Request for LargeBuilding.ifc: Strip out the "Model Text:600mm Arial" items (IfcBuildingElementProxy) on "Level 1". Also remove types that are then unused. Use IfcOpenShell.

First a look at what the model holds.

```python
import ifcopenshell
import ifcopenshell.util.element

model = ifcopenshell.open("LargeBuilding.ifc")
print(model.schema)
storey = next(s for s in model.by_type("IfcBuildingStorey") if s.Name == "Level 1")
proxies = [e for e in ifcopenshell.util.element.get_decomposition(storey) if e.is_a("IfcBuildingElementProxy")]
seen = {}
for e in proxies:
    element_type = ifcopenshell.util.element.get_type(e)
    name = element_type.Name if element_type not in (None, e) else None
    seen[name] = seen.get(name, 0) + 1
for name, count in sorted(seen.items(), key=str):
    print(count, "x", name)
```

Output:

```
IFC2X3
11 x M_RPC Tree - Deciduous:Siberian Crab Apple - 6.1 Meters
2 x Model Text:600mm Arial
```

```python
import ifcopenshell
import ifcopenshell.api.root
import ifcopenshell.util.element

model = ifcopenshell.open("LargeBuilding.ifc")

storey = next(s for s in model.by_type("IfcBuildingStorey") if s.Name == "Level 1")
proxies = [e for e in ifcopenshell.util.element.get_decomposition(storey) if e.is_a("IfcBuildingElementProxy")]
targets = [e for e in proxies if (t := ifcopenshell.util.element.get_type(e)) not in (None, e) and t.Name == "Model Text:600mm Arial"]
types = {ifcopenshell.util.element.get_type(e) for e in targets} - {None, *targets}

for e in targets:
    ifcopenshell.api.root.remove_product(model, product=e)
print(len(targets), "removed")

unused = [t for t in types if not ifcopenshell.util.element.get_types(t)]
for t in unused:
    ifcopenshell.api.root.remove_product(model, product=t)
print(len(unused), "unused types removed")

model.write("LargeBuilding_v2.ifc")
```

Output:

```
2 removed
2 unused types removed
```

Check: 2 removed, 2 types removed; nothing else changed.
